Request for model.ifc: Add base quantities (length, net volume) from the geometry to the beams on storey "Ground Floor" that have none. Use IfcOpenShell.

First a look at what the model holds.

```python
import ifcopenshell
import ifcopenshell.util.element
import ifcopenshell.util.unit

model = ifcopenshell.open("model.ifc")
print(model.schema)
for unit_type in ("LENGTHUNIT", "AREAUNIT", "VOLUMEUNIT"):
    print(unit_type, ifcopenshell.util.unit.calculate_unit_scale(model, unit_type))
storey = next(s for s in model.by_type("IfcBuildingStorey") if s.Name == "Ground Floor")
beams = [e for e in ifcopenshell.util.element.get_decomposition(storey) if e.is_a("IfcBeam")]
for e in sorted(beams, key=lambda e: e.id()):
    print(e.id(), e.is_a(), e.Name, list(ifcopenshell.util.element.get_psets(e, qtos_only=True)), sep=" | ")
```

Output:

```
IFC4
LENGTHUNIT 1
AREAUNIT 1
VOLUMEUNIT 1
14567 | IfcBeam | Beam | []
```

```python
import ifcopenshell
import ifcopenshell.api.pset
import ifcopenshell.geom
import ifcopenshell.util.element
import ifcopenshell.util.shape
import ifcopenshell.util.unit

model = ifcopenshell.open("model.ifc")
unit_scale = ifcopenshell.util.unit.calculate_unit_scale(model)
volume_scale = ifcopenshell.util.unit.calculate_unit_scale(model, "VOLUMEUNIT")
settings = ifcopenshell.geom.settings()

storey = next(s for s in model.by_type("IfcBuildingStorey") if s.Name == "Ground Floor")
beams = [e for e in ifcopenshell.util.element.get_decomposition(storey) if e.is_a("IfcBeam")]

for e in sorted(beams, key=lambda e: e.id()):
    if ifcopenshell.util.element.get_psets(e, qtos_only=True, should_inherit=False):
        continue
    # Geometry comes back in metres, in the element's own axes.
    shape = ifcopenshell.geom.create_shape(settings, e)
    values = {
        "Length": ifcopenshell.util.shape.get_max_xyz(shape.geometry) / unit_scale,
        "NetVolume": ifcopenshell.util.shape.get_volume(shape.geometry) / volume_scale,
    }
    qto = ifcopenshell.api.pset.add_qto(model, product=e, name="Qto_BeamBaseQuantities")
    ifcopenshell.api.pset.edit_qto(model, qto=qto, properties=values)
    print(e.id(), {k: round(v, 3) for k, v in values.items()})

model.write("model_rev.ifc")
```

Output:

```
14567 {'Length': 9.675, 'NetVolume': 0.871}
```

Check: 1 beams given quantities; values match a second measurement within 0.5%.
